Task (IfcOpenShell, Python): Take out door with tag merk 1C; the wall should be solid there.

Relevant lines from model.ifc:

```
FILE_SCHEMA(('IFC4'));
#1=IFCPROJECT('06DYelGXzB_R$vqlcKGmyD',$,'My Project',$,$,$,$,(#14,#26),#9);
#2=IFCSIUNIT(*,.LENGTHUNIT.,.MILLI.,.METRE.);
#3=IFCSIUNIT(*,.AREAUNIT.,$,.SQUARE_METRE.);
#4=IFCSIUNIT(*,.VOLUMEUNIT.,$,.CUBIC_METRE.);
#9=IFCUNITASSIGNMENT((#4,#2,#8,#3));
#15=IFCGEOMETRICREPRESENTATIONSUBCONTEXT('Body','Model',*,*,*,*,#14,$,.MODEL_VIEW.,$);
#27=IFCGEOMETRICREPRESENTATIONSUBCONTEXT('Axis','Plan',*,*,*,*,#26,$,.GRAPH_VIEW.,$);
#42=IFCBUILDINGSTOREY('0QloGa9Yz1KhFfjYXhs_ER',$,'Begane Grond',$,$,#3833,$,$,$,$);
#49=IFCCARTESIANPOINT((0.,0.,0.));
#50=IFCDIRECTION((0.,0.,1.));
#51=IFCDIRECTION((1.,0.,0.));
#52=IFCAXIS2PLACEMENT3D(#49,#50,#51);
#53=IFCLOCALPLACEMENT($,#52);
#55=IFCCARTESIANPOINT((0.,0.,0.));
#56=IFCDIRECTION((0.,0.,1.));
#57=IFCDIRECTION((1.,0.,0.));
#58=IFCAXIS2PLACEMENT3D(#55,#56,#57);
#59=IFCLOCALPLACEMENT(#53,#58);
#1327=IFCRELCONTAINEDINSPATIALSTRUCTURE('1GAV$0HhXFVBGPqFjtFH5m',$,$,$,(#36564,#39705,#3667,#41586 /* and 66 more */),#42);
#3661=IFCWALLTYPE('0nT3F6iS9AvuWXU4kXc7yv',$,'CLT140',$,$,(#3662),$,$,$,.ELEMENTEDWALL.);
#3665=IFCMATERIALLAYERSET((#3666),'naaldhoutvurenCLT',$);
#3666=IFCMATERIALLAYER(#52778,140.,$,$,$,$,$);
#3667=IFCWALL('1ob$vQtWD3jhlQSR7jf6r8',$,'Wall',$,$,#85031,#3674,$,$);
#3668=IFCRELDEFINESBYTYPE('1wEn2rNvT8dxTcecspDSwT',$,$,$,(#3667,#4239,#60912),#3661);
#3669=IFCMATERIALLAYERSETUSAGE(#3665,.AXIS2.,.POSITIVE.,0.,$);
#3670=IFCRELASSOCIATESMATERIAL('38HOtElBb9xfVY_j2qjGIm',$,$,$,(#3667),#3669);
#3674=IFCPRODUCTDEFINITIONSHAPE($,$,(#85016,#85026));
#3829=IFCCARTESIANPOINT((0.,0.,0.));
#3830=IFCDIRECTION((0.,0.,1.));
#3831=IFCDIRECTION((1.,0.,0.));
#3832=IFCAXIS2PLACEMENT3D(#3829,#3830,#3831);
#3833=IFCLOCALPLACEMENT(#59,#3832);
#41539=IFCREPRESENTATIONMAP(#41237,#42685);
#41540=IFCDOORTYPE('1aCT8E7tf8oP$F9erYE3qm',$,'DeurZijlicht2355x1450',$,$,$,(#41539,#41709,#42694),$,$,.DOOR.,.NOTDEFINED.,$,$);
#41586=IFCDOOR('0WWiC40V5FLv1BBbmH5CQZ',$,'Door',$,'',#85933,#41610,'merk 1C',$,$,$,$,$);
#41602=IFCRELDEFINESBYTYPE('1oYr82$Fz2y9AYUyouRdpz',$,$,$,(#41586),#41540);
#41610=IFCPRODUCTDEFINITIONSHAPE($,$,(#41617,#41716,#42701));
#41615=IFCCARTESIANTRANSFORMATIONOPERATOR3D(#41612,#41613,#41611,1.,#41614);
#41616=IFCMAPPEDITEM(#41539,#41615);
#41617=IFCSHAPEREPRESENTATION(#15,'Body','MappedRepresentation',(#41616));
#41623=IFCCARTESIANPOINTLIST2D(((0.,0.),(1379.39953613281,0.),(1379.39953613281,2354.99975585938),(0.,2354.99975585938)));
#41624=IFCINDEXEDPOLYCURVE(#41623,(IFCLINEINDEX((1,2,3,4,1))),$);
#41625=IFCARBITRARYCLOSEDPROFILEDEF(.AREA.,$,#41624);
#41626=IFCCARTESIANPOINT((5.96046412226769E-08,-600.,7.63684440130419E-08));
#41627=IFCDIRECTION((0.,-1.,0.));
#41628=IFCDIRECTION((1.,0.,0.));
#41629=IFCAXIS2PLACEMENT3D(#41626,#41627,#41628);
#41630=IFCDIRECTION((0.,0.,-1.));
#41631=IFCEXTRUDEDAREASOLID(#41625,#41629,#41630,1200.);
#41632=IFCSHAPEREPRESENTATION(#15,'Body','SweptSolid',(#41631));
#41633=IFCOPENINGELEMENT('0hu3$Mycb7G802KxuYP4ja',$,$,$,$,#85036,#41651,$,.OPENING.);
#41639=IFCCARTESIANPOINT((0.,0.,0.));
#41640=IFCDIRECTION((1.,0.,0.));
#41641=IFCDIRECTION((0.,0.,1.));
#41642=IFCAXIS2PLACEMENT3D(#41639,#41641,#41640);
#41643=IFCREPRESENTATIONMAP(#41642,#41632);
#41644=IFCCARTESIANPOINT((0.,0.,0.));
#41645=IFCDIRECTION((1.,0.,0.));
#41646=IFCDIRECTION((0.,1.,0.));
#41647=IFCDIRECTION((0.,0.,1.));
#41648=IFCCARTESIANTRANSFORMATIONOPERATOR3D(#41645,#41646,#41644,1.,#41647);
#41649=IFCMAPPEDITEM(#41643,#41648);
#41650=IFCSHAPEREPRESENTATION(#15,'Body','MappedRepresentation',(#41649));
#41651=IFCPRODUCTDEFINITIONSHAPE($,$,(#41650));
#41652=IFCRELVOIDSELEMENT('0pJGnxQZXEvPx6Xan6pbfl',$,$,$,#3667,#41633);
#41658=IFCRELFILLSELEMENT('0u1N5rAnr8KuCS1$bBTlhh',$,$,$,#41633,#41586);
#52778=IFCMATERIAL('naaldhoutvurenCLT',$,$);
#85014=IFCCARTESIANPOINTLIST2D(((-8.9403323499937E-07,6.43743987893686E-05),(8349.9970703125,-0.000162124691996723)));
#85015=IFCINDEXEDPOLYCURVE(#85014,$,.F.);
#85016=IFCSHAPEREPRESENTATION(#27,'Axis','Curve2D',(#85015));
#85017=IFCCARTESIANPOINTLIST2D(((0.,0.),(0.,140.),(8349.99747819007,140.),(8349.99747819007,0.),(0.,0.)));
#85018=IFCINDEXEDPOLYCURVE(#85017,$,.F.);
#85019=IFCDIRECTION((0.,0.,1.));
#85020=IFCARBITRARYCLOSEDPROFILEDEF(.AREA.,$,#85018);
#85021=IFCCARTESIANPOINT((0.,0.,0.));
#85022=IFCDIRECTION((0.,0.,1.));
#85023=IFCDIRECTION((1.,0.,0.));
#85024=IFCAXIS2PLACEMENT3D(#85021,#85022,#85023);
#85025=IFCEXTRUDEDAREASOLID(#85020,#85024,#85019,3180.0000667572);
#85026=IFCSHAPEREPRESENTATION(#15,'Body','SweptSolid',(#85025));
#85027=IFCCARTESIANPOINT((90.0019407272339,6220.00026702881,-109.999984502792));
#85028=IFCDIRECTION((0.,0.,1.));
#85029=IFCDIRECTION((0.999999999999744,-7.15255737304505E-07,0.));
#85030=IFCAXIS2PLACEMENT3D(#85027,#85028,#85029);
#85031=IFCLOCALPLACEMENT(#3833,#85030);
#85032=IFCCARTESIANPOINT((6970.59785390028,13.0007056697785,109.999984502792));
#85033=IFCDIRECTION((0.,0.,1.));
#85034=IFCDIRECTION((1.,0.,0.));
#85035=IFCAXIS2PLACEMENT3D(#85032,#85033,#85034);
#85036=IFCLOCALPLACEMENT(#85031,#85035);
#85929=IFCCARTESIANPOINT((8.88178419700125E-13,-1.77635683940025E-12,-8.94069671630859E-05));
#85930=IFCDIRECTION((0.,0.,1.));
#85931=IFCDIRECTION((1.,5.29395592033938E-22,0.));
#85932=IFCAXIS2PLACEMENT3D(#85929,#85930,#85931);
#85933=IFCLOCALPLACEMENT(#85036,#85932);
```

```python
import ifcopenshell
import ifcopenshell.api.feature
import ifcopenshell.api.root
import ifcopenshell.geom
import ifcopenshell.util.shape

model = ifcopenshell.open("model.ifc")
settings = ifcopenshell.geom.settings()


def volume(element):
    """Net volume in cubic metres, openings subtracted."""
    shape = ifcopenshell.geom.create_shape(settings, element)
    return ifcopenshell.util.shape.get_volume(shape.geometry)


door = model.by_guid("0WWiC40V5FLv1BBbmH5CQZ")
opening = door.FillsVoids[0].RelatingOpeningElement
wall = opening.VoidsElements[0].RelatingBuildingElement
before = volume(wall)

ifcopenshell.api.root.remove_product(model, product=door)
ifcopenshell.api.feature.remove_feature(model, feature=opening)

after = volume(wall)

print(f"wall volume {before:.3f} -> {after:.3f} m3")

model.write("model_updated.ifc")
```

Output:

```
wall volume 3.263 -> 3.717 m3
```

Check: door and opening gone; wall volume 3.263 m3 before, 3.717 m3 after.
